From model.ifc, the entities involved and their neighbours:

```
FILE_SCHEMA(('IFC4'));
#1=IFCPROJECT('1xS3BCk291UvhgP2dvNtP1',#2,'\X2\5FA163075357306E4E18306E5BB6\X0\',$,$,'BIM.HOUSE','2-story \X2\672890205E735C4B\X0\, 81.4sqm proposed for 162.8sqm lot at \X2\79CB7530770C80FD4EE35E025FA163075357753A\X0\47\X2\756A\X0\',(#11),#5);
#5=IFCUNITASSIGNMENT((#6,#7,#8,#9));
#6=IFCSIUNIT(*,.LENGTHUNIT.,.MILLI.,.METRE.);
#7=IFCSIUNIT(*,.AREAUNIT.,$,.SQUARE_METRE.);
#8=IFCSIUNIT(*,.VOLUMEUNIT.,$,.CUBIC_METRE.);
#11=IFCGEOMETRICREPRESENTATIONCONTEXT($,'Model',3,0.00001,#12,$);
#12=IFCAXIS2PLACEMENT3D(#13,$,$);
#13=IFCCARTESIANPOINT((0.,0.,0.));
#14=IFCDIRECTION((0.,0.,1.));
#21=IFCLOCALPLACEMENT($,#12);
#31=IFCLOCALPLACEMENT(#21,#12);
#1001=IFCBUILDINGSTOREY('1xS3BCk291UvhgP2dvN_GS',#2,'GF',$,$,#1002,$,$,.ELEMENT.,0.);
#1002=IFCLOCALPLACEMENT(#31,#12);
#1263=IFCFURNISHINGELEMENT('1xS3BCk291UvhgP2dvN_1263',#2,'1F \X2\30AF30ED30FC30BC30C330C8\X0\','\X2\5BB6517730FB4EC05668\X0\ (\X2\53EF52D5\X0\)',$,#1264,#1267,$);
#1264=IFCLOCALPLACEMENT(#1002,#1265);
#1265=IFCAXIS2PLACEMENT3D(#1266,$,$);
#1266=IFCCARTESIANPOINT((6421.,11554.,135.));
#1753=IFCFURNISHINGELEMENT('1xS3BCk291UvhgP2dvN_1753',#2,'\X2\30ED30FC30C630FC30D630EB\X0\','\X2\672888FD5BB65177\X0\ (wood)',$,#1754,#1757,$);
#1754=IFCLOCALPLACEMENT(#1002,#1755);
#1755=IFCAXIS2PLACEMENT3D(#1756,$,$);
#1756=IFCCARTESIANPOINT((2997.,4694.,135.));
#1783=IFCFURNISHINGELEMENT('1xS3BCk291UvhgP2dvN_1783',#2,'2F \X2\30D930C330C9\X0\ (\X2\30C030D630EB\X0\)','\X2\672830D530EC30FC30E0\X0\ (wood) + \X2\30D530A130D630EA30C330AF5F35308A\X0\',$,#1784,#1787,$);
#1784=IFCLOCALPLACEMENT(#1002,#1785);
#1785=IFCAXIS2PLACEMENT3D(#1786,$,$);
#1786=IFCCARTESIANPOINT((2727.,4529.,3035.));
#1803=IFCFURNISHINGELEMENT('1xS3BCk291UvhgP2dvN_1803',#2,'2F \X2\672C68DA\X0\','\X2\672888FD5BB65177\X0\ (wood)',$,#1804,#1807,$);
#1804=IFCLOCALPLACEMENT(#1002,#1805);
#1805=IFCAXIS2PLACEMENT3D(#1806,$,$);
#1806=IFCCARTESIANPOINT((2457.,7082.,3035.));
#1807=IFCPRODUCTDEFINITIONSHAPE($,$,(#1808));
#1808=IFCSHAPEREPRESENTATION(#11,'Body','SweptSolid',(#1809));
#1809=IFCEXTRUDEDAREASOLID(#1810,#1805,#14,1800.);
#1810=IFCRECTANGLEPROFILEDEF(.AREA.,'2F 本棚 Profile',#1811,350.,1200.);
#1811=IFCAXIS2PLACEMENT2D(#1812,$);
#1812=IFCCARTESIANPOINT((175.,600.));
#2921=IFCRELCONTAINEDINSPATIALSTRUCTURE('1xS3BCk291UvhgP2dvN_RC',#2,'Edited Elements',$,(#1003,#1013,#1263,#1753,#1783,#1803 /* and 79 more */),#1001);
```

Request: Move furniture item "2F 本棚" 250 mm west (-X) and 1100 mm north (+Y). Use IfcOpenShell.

```python
import ifcopenshell
import ifcopenshell.api.geometry
import ifcopenshell.util.placement
import ifcopenshell.util.unit

model = ifcopenshell.open("model.ifc")
unit_scale = ifcopenshell.util.unit.calculate_unit_scale(model)

item = model.by_guid("1xS3BCk291UvhgP2dvN_1803")
matrix = ifcopenshell.util.placement.get_local_placement(item.ObjectPlacement)
matrix[0, 3] -= 0.25 / unit_scale
matrix[1, 3] += 1.1 / unit_scale
ifcopenshell.api.geometry.edit_object_placement(model, product=item, matrix=matrix, is_si=False)

print(ifcopenshell.util.placement.get_local_placement(item.ObjectPlacement).round(3) + 0.0)

model.write("model_rev.ifc")
```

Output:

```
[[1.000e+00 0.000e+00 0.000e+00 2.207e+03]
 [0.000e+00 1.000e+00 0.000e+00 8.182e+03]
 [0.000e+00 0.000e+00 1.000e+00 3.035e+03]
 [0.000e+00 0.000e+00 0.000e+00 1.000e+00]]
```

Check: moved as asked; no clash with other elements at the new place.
